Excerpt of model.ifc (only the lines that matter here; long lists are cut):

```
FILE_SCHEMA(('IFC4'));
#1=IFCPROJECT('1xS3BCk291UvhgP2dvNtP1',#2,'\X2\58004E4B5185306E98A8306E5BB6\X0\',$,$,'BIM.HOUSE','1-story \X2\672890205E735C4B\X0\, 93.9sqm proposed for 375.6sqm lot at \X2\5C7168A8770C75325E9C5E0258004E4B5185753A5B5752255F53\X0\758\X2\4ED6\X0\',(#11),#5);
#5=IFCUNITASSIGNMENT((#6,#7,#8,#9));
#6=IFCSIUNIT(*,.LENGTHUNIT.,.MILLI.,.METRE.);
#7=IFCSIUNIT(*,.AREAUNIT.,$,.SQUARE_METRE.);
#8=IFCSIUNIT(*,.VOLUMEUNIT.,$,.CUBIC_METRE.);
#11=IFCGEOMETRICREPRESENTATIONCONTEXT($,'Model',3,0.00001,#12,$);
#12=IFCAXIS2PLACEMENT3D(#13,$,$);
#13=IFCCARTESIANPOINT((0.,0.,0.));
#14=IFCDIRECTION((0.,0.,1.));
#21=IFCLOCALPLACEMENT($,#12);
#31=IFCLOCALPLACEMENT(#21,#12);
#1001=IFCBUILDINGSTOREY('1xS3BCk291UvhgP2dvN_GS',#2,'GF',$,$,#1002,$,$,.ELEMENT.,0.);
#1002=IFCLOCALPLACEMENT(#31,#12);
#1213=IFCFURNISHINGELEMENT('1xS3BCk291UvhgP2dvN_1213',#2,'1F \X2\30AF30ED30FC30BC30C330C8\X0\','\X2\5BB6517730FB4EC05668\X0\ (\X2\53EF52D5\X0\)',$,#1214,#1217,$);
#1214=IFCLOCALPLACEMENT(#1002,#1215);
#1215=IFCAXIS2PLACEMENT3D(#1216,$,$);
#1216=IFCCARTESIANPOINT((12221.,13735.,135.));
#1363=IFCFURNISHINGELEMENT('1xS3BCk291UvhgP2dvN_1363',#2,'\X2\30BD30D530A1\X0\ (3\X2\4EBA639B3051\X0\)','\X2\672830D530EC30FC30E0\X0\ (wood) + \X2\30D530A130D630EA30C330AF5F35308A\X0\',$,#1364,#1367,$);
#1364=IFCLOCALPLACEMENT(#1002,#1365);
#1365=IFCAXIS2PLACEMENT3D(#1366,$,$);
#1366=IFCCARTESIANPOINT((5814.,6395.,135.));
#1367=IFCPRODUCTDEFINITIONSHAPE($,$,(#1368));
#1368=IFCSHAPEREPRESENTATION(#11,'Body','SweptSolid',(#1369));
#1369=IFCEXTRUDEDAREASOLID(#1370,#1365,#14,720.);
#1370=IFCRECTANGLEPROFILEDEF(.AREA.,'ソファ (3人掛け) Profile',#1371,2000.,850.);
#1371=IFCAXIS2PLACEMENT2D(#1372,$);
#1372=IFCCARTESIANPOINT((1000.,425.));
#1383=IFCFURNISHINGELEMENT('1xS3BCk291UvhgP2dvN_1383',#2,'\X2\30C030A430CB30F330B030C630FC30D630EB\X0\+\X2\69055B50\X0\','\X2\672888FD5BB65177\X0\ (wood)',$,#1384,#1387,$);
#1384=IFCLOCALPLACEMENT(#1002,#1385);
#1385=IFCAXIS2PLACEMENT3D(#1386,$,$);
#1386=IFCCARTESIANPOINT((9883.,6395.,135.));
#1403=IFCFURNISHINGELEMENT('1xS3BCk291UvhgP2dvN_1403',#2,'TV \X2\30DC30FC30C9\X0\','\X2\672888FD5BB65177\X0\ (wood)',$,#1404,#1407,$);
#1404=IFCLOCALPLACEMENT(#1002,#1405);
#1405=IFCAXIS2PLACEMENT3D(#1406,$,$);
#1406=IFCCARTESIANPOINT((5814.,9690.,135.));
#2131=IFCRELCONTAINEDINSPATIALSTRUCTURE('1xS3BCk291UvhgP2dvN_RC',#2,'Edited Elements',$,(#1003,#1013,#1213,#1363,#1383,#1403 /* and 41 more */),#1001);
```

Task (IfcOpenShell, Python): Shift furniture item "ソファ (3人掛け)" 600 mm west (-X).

```python
import ifcopenshell
import ifcopenshell.api.geometry
import ifcopenshell.util.placement
import ifcopenshell.util.unit

model = ifcopenshell.open("model.ifc")
unit_scale = ifcopenshell.util.unit.calculate_unit_scale(model)

item = model.by_id(1363)
matrix = ifcopenshell.util.placement.get_local_placement(item.ObjectPlacement)
matrix[0, 3] -= 0.6 / unit_scale
ifcopenshell.api.geometry.edit_object_placement(model, product=item, matrix=matrix, is_si=False)

print(ifcopenshell.util.placement.get_local_placement(item.ObjectPlacement).round(3) + 0.0)

model.write("model_updated.ifc")
```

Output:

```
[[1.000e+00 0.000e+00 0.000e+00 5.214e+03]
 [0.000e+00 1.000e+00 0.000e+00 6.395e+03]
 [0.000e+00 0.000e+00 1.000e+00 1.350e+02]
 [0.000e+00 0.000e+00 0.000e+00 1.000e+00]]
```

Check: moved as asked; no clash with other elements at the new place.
